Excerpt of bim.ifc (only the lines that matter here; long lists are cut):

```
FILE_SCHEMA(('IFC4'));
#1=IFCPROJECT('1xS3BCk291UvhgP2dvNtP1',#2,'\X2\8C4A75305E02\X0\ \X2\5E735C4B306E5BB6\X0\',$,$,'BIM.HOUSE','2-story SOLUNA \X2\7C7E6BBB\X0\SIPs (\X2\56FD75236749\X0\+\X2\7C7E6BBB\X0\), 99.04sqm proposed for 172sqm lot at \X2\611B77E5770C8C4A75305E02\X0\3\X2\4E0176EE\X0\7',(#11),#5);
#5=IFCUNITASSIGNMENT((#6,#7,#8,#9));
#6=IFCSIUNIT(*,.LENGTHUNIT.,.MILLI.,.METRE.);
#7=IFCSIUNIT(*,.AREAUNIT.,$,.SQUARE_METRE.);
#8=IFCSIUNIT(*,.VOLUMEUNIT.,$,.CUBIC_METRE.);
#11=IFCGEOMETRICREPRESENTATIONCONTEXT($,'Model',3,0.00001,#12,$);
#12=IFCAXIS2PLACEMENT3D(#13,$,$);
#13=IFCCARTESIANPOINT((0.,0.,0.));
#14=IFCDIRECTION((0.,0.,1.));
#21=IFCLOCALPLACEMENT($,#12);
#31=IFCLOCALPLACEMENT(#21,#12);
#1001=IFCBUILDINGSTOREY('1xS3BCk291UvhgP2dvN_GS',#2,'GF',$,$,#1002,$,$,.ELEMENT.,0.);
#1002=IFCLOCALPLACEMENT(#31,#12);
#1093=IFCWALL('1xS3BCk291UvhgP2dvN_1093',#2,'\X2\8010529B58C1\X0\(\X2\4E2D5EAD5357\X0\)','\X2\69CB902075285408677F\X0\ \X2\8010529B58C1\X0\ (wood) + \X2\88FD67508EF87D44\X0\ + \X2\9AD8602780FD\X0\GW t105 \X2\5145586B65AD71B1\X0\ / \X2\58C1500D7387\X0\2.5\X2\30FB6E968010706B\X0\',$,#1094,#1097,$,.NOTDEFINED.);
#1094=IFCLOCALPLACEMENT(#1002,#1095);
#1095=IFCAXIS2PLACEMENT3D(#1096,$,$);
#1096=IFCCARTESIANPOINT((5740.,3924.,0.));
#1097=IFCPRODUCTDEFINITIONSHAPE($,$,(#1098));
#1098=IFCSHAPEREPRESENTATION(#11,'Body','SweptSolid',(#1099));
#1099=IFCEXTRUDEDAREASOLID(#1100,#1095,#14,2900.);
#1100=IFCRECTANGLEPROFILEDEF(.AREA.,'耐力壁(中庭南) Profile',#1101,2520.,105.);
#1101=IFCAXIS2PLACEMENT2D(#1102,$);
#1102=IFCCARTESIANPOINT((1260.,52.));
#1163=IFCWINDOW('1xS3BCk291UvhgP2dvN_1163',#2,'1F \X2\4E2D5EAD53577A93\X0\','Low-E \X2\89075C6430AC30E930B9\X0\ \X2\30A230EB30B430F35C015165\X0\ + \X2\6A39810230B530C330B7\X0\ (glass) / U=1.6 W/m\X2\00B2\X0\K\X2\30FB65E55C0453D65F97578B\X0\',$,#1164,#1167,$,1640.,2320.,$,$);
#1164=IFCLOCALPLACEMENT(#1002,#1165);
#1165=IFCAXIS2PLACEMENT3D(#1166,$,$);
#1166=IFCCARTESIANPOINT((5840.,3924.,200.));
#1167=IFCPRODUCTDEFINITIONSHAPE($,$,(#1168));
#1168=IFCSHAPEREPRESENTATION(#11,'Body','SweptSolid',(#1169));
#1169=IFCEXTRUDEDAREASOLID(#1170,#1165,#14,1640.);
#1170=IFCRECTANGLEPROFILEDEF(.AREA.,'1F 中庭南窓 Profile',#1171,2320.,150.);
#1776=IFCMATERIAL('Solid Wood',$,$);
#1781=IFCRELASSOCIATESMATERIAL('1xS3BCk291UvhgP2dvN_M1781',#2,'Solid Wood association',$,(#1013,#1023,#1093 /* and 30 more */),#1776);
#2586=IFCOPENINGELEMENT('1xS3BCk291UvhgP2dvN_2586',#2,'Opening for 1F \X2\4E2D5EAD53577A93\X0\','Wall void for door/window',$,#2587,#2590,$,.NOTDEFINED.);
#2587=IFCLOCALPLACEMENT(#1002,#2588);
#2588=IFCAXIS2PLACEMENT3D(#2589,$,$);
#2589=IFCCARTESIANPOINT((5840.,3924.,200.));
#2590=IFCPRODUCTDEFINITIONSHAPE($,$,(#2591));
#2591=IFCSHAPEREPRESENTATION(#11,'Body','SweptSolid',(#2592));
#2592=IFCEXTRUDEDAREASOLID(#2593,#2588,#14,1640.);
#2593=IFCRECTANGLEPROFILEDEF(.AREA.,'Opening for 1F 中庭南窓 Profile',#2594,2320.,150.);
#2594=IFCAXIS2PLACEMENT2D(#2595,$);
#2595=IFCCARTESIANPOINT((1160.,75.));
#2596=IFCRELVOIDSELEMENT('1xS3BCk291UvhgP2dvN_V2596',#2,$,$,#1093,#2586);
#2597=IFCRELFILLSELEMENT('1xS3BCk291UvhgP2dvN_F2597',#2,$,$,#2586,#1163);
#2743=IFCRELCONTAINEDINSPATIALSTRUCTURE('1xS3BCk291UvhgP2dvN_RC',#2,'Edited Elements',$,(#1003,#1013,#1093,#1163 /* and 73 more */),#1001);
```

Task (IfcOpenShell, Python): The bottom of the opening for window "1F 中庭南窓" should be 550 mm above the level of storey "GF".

```python
import numpy as np
import ifcopenshell
import ifcopenshell.api.geometry
import ifcopenshell.geom
import ifcopenshell.util.element
import ifcopenshell.util.placement
import ifcopenshell.util.shape
import ifcopenshell.util.unit

model = ifcopenshell.open("bim.ifc")
unit_scale = ifcopenshell.util.unit.calculate_unit_scale(model)

window = model.by_guid("1xS3BCk291UvhgP2dvN_1163")
opening = window.FillsVoids[0].RelatingOpeningElement
storey = ifcopenshell.util.element.get_container(window, ifc_class="IfcBuildingStorey")
level = ifcopenshell.util.placement.get_local_placement(storey.ObjectPlacement)[2, 3]

# The opening's origin need not be at the sill, so measure its lowest point.
shape = ifcopenshell.geom.create_shape(ifcopenshell.geom.settings(), opening)
bottom = ifcopenshell.util.shape.get_shape_bottom_elevation(shape, shape.geometry) / unit_scale
dz = level + 0.55 / unit_scale - bottom

shift = np.array([0.0, 0.0, dz])
# The window is not placed relative to its opening, so move both.
for product in (opening, window):
    matrix = ifcopenshell.util.placement.get_local_placement(product.ObjectPlacement)
    matrix[:3, 3] += shift
    ifcopenshell.api.geometry.edit_object_placement(model, product=product, matrix=matrix, is_si=False)

print(f"moved by {dz * unit_scale:+.3f} m")

model.write("bim-out.ifc")
```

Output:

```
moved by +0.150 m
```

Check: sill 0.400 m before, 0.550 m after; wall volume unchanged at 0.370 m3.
